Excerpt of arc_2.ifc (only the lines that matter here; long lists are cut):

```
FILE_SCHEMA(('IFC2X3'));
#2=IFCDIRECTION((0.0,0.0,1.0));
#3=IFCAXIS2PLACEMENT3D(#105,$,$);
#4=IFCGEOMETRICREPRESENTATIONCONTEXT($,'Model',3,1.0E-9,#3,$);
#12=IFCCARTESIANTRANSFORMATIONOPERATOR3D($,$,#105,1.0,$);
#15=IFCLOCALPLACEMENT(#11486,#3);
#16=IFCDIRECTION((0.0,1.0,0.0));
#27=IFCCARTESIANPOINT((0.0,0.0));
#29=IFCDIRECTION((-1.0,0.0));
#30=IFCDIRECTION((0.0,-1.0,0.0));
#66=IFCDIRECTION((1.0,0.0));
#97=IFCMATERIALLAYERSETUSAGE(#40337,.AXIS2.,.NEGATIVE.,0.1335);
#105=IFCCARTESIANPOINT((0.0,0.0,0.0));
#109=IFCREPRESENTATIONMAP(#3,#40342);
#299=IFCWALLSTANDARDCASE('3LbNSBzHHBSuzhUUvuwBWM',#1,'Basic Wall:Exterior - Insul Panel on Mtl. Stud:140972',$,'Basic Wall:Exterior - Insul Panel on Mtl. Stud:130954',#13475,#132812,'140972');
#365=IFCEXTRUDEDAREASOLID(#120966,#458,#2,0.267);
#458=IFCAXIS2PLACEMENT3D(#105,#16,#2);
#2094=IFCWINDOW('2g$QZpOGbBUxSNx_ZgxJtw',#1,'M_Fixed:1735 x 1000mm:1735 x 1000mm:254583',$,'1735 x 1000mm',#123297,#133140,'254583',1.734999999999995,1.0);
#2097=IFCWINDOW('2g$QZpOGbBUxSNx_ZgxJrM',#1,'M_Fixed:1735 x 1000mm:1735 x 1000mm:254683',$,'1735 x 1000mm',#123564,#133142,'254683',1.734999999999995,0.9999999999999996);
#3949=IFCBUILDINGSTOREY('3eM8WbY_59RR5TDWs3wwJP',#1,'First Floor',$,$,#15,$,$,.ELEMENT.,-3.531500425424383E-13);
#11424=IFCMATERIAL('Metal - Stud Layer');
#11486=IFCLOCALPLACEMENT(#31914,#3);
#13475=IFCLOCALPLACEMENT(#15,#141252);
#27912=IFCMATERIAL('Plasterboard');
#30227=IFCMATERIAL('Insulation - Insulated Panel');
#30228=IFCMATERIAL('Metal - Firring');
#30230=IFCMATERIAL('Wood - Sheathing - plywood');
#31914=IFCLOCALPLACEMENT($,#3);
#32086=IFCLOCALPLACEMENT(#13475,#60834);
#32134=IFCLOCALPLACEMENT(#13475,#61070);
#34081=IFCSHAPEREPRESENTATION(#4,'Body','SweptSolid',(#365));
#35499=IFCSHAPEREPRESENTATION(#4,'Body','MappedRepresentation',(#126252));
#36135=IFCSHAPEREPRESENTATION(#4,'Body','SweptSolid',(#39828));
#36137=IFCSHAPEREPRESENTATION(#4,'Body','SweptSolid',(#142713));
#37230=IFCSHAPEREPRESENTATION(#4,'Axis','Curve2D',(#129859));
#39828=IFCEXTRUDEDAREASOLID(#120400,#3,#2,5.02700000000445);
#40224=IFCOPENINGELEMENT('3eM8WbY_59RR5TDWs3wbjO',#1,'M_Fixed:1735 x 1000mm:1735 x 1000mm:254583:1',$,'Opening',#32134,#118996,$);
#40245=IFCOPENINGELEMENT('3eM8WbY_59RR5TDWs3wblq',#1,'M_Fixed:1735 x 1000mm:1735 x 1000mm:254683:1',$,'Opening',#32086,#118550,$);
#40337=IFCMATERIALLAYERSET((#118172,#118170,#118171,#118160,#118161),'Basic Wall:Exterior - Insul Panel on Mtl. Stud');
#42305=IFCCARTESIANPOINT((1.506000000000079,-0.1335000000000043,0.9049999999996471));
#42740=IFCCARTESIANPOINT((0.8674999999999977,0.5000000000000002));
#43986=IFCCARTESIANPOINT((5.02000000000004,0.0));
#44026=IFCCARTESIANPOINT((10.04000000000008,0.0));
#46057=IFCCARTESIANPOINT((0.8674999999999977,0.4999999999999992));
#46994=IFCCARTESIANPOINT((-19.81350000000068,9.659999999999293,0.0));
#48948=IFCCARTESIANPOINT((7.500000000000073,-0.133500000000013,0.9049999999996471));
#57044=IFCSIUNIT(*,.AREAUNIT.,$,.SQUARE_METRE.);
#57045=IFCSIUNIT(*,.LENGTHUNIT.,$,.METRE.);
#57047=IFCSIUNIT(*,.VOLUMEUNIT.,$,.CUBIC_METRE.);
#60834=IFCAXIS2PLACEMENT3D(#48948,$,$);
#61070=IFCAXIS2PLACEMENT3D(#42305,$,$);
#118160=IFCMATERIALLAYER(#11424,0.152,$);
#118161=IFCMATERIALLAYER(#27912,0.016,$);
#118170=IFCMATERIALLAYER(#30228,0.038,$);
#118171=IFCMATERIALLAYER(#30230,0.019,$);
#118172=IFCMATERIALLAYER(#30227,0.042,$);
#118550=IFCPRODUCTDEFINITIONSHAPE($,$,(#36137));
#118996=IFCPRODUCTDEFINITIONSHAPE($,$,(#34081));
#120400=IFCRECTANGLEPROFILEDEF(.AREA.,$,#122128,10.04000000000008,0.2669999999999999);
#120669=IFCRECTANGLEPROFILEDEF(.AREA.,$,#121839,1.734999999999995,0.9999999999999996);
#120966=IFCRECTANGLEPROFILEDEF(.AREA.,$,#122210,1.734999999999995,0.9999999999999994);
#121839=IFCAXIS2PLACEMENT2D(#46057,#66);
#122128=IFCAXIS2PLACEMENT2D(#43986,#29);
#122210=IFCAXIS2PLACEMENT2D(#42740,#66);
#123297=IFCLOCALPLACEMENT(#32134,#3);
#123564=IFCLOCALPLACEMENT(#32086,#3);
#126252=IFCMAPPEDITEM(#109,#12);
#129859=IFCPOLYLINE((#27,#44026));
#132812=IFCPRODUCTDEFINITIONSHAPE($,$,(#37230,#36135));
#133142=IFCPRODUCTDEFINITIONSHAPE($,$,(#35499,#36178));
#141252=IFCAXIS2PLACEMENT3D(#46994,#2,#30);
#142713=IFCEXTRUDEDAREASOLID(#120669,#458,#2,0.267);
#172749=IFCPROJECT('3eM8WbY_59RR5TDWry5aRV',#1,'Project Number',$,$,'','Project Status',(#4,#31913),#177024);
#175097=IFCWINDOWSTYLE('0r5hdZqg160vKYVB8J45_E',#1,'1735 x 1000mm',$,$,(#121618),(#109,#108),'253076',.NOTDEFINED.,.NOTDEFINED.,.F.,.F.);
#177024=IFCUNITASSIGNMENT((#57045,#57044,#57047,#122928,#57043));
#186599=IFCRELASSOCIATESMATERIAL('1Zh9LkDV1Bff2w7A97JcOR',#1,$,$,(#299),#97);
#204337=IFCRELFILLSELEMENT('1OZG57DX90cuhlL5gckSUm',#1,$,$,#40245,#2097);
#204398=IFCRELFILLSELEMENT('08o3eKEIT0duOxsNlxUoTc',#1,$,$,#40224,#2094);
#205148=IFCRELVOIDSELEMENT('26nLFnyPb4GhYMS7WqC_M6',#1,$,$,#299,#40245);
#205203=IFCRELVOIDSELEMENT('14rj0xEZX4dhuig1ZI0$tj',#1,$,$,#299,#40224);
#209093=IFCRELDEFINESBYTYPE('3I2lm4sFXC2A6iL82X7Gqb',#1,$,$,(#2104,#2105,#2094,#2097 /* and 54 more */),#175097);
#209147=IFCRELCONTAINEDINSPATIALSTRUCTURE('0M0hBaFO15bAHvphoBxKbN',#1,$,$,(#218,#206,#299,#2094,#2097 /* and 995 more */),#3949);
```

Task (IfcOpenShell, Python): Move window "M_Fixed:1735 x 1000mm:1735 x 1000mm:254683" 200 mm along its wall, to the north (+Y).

```python
import ifcopenshell
import ifcopenshell.api.geometry
import ifcopenshell.util.placement
import ifcopenshell.util.unit

model = ifcopenshell.open("arc_2.ifc")
unit_scale = ifcopenshell.util.unit.calculate_unit_scale(model)

window = model.by_guid("2g$QZpOGbBUxSNx_ZgxJrM")
opening = window.FillsVoids[0].RelatingOpeningElement
wall = opening.VoidsElements[0].RelatingBuildingElement

wall_matrix = ifcopenshell.util.placement.get_local_placement(wall.ObjectPlacement)
shift = wall_matrix[:3, 0] * -0.2 / unit_scale
before = ifcopenshell.util.placement.get_local_placement(window.ObjectPlacement)[:3, 3].copy()

# The window is placed relative to its opening, so it follows when the opening moves.
matrix = ifcopenshell.util.placement.get_local_placement(opening.ObjectPlacement)
matrix[:3, 3] += shift
ifcopenshell.api.geometry.edit_object_placement(
    model, product=opening, matrix=matrix, is_si=False, should_transform_children=True
)

after = ifcopenshell.util.placement.get_local_placement(window.ObjectPlacement)[:3, 3]
print("window moved by", (after - before).round(3) + 0.0)

model.write("arc_2_v2.ifc")
```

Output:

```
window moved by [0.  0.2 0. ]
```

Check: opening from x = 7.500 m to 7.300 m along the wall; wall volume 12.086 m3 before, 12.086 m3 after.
